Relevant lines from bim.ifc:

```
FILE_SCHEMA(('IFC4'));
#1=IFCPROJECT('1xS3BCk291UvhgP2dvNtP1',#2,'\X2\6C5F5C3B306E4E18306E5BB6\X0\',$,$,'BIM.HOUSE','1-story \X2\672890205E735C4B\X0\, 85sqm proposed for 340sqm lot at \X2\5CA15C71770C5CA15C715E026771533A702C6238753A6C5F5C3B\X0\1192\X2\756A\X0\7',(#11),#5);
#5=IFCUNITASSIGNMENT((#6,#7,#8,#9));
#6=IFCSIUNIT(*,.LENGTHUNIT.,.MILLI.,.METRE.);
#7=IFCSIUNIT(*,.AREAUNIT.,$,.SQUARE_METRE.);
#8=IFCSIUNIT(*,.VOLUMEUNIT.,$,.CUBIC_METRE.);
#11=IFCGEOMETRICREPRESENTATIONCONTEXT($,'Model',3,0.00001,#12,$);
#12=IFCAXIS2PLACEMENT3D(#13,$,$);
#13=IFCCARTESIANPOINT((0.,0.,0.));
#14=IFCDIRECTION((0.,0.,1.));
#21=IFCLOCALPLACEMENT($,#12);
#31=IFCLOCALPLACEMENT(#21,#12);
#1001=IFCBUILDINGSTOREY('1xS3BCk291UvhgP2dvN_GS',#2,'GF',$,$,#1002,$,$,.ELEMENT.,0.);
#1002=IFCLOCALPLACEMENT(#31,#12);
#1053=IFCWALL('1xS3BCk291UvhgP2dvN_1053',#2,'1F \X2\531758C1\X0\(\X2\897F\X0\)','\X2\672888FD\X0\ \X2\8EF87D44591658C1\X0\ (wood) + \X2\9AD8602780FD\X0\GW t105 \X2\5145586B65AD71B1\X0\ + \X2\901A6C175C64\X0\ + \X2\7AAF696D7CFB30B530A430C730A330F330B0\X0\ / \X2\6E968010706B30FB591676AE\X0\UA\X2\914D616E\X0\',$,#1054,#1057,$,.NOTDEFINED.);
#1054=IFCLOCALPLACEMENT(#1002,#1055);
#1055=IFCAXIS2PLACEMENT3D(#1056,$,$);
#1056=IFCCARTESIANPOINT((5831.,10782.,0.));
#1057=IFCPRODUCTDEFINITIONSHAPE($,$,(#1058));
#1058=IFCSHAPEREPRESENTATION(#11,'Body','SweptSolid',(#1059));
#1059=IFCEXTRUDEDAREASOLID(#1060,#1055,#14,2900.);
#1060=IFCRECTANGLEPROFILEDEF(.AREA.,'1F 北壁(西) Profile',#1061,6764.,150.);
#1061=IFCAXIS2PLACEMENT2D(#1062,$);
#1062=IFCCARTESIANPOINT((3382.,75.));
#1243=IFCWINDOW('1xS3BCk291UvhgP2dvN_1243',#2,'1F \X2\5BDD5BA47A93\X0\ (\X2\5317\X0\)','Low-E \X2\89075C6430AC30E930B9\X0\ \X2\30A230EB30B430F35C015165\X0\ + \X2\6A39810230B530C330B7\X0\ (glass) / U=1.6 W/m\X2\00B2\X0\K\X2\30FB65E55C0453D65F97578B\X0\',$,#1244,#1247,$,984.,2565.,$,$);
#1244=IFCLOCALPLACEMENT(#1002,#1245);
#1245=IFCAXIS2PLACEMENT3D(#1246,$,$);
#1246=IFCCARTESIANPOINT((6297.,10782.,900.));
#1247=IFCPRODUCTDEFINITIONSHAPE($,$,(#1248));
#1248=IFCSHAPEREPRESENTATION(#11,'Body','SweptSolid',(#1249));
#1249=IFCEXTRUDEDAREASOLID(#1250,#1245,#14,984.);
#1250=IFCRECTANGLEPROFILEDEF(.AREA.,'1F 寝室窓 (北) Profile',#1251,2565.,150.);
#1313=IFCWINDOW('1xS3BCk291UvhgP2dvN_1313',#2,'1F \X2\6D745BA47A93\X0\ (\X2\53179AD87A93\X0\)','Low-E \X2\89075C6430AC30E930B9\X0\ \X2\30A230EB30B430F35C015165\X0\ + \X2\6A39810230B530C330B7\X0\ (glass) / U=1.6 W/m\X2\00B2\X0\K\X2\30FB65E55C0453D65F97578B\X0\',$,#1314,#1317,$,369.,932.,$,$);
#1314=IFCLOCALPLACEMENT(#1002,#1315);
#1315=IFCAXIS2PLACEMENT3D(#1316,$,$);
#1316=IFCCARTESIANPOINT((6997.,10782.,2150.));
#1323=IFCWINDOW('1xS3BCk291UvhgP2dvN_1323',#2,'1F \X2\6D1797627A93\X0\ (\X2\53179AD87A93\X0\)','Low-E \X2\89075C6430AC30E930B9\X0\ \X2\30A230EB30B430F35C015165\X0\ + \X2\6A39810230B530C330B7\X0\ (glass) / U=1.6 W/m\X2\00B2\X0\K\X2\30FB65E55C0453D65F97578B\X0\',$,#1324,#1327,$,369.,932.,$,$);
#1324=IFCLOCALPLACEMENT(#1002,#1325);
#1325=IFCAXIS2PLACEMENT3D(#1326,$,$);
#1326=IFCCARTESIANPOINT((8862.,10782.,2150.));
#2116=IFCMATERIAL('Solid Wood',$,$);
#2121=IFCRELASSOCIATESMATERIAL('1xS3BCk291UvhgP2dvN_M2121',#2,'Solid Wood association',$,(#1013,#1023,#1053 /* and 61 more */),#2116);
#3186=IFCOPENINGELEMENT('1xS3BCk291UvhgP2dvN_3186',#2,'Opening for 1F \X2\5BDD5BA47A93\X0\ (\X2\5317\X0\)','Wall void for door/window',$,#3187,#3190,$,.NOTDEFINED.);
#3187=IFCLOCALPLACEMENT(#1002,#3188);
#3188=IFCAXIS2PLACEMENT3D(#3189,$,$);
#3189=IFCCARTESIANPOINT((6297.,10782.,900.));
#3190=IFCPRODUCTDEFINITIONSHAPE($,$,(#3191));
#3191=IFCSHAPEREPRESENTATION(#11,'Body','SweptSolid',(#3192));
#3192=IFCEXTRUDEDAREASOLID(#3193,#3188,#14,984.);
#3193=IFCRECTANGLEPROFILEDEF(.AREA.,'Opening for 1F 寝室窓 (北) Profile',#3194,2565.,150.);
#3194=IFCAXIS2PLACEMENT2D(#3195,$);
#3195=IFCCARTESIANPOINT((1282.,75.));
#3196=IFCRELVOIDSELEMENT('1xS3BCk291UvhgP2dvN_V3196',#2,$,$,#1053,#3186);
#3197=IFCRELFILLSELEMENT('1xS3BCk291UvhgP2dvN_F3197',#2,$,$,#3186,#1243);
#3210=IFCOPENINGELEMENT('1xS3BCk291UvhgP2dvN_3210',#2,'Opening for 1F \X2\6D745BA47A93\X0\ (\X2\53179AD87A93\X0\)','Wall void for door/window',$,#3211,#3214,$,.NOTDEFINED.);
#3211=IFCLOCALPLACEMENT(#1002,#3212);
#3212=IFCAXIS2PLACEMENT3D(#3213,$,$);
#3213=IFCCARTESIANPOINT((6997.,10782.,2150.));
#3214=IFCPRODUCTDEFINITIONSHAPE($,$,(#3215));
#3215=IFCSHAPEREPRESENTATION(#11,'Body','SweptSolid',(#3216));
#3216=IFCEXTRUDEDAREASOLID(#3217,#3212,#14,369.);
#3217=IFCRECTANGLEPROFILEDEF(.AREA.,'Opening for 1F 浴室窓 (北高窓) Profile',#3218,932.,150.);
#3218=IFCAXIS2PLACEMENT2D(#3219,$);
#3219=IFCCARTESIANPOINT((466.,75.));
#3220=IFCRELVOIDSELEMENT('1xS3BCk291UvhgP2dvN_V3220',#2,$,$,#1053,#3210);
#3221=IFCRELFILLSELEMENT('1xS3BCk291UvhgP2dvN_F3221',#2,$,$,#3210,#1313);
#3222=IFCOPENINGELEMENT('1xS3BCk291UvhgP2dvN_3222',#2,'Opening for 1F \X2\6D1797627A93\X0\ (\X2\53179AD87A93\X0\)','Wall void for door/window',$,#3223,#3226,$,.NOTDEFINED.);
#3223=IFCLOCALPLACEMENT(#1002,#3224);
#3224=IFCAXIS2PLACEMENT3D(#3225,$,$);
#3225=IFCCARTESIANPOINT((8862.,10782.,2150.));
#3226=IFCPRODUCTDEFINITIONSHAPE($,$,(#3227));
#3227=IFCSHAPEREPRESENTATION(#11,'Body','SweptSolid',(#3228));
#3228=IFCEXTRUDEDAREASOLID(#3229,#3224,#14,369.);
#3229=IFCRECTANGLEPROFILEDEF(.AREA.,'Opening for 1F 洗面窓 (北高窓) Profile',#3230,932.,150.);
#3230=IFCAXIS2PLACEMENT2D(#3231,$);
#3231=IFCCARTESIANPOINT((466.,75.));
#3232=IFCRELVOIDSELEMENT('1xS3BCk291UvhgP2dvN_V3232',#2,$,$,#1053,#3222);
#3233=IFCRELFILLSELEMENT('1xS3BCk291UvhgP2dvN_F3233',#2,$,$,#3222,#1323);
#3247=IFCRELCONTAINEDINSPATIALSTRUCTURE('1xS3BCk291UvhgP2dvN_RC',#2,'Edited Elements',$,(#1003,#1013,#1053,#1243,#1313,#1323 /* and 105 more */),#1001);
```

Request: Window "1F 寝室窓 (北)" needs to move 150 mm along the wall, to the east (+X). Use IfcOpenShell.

```python
import ifcopenshell
import ifcopenshell.api.geometry
import ifcopenshell.util.placement
import ifcopenshell.util.unit

model = ifcopenshell.open("bim.ifc")
unit_scale = ifcopenshell.util.unit.calculate_unit_scale(model)

window = model.by_guid("1xS3BCk291UvhgP2dvN_1243")
opening = window.FillsVoids[0].RelatingOpeningElement
wall = opening.VoidsElements[0].RelatingBuildingElement

wall_matrix = ifcopenshell.util.placement.get_local_placement(wall.ObjectPlacement)
shift = wall_matrix[:3, 0] * 0.15 / unit_scale
before = ifcopenshell.util.placement.get_local_placement(window.ObjectPlacement)[:3, 3].copy()

# The window is not placed relative to its opening, so move both.
for product in (opening, window):
    matrix = ifcopenshell.util.placement.get_local_placement(product.ObjectPlacement)
    matrix[:3, 3] += shift
    ifcopenshell.api.geometry.edit_object_placement(model, product=product, matrix=matrix, is_si=False)

after = ifcopenshell.util.placement.get_local_placement(window.ObjectPlacement)[:3, 3]
print("window moved by", (after - before).round(3) + 0.0)

model.write("bim_edited.ifc")
```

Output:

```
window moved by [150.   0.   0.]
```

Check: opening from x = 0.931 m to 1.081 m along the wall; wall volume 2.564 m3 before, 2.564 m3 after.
